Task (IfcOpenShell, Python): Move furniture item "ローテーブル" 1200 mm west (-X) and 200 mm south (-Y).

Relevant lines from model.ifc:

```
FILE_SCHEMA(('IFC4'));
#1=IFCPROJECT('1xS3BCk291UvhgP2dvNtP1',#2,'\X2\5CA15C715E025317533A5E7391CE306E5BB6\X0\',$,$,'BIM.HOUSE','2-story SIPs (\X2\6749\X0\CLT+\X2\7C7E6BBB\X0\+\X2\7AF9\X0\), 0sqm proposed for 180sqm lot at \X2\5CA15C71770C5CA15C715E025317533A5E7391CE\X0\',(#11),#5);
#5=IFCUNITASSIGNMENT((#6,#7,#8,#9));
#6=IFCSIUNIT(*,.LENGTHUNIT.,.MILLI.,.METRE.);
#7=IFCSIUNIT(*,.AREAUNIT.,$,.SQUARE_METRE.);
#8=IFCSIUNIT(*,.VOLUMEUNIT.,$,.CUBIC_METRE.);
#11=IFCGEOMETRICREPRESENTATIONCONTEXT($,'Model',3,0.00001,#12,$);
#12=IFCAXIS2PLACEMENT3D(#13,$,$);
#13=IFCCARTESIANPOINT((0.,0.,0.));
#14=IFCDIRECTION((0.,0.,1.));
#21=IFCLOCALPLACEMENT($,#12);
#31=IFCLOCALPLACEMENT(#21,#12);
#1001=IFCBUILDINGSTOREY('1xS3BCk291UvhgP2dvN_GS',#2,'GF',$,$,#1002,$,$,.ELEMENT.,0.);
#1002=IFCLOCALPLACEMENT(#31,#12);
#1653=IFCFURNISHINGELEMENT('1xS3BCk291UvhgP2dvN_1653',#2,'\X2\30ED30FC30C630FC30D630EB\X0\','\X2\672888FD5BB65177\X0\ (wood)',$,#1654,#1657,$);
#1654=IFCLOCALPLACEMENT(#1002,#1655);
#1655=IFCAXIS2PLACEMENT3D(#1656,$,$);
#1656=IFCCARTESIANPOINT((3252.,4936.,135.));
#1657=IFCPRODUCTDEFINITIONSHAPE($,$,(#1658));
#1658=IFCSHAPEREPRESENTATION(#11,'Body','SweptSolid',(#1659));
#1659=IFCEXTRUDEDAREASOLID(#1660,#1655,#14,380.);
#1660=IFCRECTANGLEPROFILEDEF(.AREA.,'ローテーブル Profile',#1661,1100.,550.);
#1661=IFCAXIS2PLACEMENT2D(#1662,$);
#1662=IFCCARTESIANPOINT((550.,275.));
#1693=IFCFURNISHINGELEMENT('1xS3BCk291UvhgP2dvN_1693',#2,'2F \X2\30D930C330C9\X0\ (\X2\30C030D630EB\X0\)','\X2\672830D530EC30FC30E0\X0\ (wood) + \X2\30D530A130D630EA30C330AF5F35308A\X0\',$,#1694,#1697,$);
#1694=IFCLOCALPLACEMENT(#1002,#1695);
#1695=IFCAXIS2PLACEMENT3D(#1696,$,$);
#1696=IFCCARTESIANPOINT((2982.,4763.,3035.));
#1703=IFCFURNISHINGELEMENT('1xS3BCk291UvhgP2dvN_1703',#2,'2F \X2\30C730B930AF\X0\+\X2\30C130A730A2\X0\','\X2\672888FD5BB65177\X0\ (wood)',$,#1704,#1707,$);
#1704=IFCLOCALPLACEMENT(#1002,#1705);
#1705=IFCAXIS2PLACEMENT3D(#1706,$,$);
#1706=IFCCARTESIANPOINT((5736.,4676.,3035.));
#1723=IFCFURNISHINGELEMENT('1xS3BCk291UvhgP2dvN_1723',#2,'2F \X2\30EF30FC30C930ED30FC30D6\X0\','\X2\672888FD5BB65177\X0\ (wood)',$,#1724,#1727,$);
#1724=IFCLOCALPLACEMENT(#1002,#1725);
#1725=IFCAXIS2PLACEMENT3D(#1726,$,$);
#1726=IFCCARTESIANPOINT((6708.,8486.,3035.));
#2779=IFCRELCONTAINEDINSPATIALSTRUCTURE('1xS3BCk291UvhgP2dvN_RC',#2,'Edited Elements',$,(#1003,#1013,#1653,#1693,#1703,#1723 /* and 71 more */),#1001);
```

```python
import ifcopenshell
import ifcopenshell.api.geometry
import ifcopenshell.util.placement

model = ifcopenshell.open("model.ifc")

item = model.by_guid("1xS3BCk291UvhgP2dvN_1653")
matrix = ifcopenshell.util.placement.get_local_placement(item.ObjectPlacement)
matrix[0, 3] -= 1200.0
matrix[1, 3] -= 200.0
ifcopenshell.api.geometry.edit_object_placement(model, product=item, matrix=matrix, is_si=False)

print(ifcopenshell.util.placement.get_local_placement(item.ObjectPlacement).round(3) + 0.0)

model.write("model_updated.ifc")
```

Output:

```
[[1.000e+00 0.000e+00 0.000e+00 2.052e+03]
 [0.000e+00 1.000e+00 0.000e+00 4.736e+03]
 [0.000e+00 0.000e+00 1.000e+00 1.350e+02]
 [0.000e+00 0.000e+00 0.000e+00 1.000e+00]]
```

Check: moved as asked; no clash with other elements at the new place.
